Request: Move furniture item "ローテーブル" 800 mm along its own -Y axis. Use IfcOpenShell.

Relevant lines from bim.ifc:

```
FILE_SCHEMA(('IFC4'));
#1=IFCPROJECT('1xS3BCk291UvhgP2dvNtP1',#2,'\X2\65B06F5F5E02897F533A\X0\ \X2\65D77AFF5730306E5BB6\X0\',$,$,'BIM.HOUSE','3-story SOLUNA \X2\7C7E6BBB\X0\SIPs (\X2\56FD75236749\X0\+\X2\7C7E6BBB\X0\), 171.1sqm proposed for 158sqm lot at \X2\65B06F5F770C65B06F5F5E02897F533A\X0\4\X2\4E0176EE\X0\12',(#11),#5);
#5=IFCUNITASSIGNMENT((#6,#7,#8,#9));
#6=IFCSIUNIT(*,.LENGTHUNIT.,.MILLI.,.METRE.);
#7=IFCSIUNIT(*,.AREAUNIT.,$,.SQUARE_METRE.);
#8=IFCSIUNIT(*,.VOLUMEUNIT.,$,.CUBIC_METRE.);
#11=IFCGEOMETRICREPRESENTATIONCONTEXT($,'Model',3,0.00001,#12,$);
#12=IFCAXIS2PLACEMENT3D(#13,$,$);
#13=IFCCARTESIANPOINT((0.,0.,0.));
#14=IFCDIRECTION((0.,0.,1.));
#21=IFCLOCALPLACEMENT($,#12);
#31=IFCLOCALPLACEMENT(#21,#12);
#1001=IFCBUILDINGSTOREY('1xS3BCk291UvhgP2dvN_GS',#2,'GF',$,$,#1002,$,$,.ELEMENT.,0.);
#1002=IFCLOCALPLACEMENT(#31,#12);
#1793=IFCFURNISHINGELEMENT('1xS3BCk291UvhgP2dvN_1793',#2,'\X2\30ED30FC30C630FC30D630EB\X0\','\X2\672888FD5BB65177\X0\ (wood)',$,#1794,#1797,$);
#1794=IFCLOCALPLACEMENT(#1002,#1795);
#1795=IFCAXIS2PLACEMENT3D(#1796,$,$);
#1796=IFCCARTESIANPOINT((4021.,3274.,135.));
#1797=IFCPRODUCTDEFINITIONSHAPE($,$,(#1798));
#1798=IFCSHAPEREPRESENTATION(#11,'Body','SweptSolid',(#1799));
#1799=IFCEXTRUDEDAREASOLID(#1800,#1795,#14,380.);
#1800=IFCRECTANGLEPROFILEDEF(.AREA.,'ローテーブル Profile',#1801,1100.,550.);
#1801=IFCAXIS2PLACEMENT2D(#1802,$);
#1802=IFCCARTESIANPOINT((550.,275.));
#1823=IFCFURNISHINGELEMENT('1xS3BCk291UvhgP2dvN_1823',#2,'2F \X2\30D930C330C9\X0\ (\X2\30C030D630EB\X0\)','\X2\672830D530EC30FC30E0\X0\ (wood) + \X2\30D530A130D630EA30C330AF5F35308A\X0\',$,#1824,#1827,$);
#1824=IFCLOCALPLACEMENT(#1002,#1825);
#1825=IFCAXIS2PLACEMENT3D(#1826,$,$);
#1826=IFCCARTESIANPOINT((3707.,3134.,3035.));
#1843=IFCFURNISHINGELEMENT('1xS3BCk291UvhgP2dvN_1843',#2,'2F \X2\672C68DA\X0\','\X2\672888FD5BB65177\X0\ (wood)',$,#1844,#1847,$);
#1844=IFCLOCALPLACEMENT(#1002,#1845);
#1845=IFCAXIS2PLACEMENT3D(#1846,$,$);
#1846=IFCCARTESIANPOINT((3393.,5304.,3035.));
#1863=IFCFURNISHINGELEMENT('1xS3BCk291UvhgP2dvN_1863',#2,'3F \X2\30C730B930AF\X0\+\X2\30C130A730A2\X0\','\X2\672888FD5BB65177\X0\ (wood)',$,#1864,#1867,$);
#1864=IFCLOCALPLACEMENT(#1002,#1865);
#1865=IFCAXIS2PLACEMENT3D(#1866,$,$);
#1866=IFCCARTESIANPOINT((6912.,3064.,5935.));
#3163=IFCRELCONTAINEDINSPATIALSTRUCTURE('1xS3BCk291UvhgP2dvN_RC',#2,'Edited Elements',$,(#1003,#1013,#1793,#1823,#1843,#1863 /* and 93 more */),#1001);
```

```python
import ifcopenshell
import ifcopenshell.api.geometry
import ifcopenshell.util.placement
import ifcopenshell.util.unit

model = ifcopenshell.open("bim.ifc")
unit_scale = ifcopenshell.util.unit.calculate_unit_scale(model)

item = model.by_guid("1xS3BCk291UvhgP2dvN_1793")
matrix = ifcopenshell.util.placement.get_local_placement(item.ObjectPlacement)
matrix[:3, 3] -= matrix[:3, 1] * 0.8 / unit_scale
ifcopenshell.api.geometry.edit_object_placement(model, product=item, matrix=matrix, is_si=False)

print(ifcopenshell.util.placement.get_local_placement(item.ObjectPlacement).round(3) + 0.0)

model.write("bim_v2.ifc")
```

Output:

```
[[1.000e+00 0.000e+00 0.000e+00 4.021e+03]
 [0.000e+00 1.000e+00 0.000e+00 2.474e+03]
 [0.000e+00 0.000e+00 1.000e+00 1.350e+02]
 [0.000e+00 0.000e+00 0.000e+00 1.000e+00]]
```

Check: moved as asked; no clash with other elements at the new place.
